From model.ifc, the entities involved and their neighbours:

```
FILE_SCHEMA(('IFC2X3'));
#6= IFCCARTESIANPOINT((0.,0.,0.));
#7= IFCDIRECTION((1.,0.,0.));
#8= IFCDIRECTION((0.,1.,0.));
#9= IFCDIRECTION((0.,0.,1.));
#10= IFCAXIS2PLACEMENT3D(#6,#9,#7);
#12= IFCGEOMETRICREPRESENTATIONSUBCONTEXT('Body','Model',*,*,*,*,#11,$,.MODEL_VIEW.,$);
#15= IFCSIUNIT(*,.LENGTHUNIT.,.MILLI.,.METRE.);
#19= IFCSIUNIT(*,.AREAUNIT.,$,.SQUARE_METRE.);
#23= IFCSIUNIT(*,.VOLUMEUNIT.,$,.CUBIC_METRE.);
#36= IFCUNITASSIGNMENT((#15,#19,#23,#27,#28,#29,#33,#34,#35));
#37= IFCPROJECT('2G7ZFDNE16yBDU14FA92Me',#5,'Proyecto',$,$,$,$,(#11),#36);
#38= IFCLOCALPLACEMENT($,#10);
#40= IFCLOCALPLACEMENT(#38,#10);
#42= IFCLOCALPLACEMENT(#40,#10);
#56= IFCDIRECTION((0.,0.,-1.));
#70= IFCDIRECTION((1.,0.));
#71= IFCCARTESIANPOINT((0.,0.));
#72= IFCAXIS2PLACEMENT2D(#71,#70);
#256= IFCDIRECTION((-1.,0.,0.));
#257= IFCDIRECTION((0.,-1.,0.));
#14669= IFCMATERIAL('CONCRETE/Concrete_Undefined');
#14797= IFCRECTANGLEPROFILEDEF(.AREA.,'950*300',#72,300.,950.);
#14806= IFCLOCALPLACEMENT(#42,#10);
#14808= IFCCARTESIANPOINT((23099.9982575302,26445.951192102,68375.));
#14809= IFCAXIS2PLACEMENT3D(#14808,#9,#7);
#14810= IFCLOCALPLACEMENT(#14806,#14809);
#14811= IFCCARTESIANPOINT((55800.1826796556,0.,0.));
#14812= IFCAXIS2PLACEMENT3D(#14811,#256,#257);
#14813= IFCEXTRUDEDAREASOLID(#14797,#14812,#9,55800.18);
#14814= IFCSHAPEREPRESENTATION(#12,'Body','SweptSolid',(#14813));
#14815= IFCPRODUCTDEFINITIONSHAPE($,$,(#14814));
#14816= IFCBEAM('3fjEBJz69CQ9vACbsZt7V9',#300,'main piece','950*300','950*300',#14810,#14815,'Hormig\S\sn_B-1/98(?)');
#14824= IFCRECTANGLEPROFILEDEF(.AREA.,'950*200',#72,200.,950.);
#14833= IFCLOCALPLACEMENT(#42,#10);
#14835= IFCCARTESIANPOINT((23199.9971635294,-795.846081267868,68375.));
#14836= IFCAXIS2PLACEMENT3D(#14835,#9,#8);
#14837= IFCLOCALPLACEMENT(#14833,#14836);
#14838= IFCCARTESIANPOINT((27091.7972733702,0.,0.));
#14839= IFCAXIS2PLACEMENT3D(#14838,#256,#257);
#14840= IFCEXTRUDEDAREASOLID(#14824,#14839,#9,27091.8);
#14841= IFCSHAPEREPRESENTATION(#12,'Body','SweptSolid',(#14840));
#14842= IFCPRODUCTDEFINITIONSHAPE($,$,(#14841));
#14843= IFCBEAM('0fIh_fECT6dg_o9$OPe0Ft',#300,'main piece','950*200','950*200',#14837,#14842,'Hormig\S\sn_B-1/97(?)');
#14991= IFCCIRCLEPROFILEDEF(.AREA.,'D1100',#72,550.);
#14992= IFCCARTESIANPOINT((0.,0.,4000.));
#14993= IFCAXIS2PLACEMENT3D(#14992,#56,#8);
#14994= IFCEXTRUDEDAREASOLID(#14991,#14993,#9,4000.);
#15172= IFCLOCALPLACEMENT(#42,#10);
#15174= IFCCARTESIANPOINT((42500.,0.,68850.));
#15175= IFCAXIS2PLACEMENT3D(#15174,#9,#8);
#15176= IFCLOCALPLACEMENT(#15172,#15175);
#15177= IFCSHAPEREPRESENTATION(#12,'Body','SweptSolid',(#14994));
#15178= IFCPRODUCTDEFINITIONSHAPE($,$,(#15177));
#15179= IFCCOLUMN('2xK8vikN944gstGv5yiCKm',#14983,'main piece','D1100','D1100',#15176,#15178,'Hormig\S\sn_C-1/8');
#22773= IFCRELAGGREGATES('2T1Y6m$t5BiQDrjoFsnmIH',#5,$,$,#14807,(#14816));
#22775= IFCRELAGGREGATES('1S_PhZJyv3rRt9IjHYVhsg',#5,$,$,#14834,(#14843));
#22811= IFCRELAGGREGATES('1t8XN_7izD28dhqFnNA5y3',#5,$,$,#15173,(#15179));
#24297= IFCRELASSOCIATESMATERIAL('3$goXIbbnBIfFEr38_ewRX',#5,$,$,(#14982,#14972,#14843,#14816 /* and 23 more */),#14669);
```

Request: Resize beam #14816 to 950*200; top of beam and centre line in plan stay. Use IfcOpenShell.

```python
import ifcopenshell
import ifcopenshell.util.element
import ifcopenshell.util.representation

model = ifcopenshell.open("model.ifc")

member = model.by_guid("3fjEBJz69CQ9vACbsZt7V9")
source = next(p for p in model.by_type("IfcRectangleProfileDef") if p.ProfileName == "950*200")

body = ifcopenshell.util.representation.get_representation(member, "Model", "Body")
solid = body.Items[0]
old_profile = solid.SweptArea

# Copy the section's sizes but keep this member's own profile position.
profile = ifcopenshell.util.element.copy(model, source)
# Profiles are centred, so shift by half the change in depth to hold the top.
shift = (old_profile.YDim - profile.YDim) / 2
x, y = old_profile.Position.Location.Coordinates
up = (0.0, 1.0)  # upwards, in the solid's own plane
location = model.createIfcCartesianPoint((x + up[0] * shift, y + up[1] * shift))
profile.Position = model.createIfcAxis2Placement2D(location, old_profile.Position.RefDirection)
solid.SweptArea = profile
if not model.get_total_inverses(old_profile):
    ifcopenshell.util.element.remove_deep2(model, old_profile)
member.Description = member.Description.replace("950*300", "950*200")
member.ObjectType = member.ObjectType.replace("950*300", "950*200")

print(solid.SweptArea)

model.write("model_v2.ifc")
```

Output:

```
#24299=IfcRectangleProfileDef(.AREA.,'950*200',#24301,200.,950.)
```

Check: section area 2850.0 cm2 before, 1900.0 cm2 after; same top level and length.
